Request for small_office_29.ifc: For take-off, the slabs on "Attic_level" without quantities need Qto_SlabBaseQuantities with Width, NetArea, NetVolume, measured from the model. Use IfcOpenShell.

First a look at what the model holds.

```python
import ifcopenshell
import ifcopenshell.util.element
import ifcopenshell.util.unit

model = ifcopenshell.open("small_office_29.ifc")
print(model.schema)
for unit_type in ("LENGTHUNIT", "AREAUNIT", "VOLUMEUNIT"):
    print(unit_type, ifcopenshell.util.unit.calculate_unit_scale(model, unit_type))
storey = next(s for s in model.by_type("IfcBuildingStorey") if s.Name == "Attic_level")
slabs = [e for e in ifcopenshell.util.element.get_decomposition(storey) if e.is_a("IfcSlab")]
for e in sorted(slabs, key=lambda e: e.id()):
    print(e.id(), e.is_a(), e.Name, list(ifcopenshell.util.element.get_psets(e, qtos_only=True)), sep=" | ")
```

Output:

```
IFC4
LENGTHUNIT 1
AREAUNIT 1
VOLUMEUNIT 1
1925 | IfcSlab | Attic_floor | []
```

```python
import ifcopenshell
import ifcopenshell.api.pset
import ifcopenshell.geom
import ifcopenshell.util.element
import ifcopenshell.util.shape
import ifcopenshell.util.unit

model = ifcopenshell.open("small_office_29.ifc")
unit_scale = ifcopenshell.util.unit.calculate_unit_scale(model)
area_scale = ifcopenshell.util.unit.calculate_unit_scale(model, "AREAUNIT")
volume_scale = ifcopenshell.util.unit.calculate_unit_scale(model, "VOLUMEUNIT")
settings = ifcopenshell.geom.settings()

storey = next(s for s in model.by_type("IfcBuildingStorey") if s.Name == "Attic_level")
slabs = [e for e in ifcopenshell.util.element.get_decomposition(storey) if e.is_a("IfcSlab")]

for e in sorted(slabs, key=lambda e: e.id()):
    if ifcopenshell.util.element.get_psets(e, qtos_only=True, should_inherit=False):
        continue
    # Geometry comes back in metres, in the element's own axes.
    shape = ifcopenshell.geom.create_shape(settings, e)
    values = {
        "Width": ifcopenshell.util.shape.get_z(shape.geometry) / unit_scale,
        "NetArea": ifcopenshell.util.shape.get_footprint_area(shape.geometry) / area_scale,
        "NetVolume": ifcopenshell.util.shape.get_volume(shape.geometry) / volume_scale,
    }
    qto = ifcopenshell.api.pset.add_qto(model, product=e, name="Qto_SlabBaseQuantities")
    ifcopenshell.api.pset.edit_qto(model, qto=qto, properties=values)
    print(e.id(), {k: round(v, 3) for k, v in values.items()})

model.write("small_office_29_rev.ifc")
```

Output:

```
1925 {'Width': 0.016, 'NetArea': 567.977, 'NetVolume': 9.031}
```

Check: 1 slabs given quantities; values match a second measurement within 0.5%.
